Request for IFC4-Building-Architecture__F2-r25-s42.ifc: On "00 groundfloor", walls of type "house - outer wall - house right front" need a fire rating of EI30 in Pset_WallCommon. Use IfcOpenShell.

First a look at what the model holds.

```python
import ifcopenshell
import ifcopenshell.util.element

model = ifcopenshell.open("IFC4-Building-Architecture__F2-r25-s42.ifc")
print(model.schema)
storey = next(s for s in model.by_type("IfcBuildingStorey") if s.Name == "00 groundfloor")
walls = [e for e in ifcopenshell.util.element.get_decomposition(storey) if e.is_a("IfcWall")]
seen = {}
for e in walls:
    element_type = ifcopenshell.util.element.get_type(e)
    key = (element_type.Name if element_type != e and element_type else None, ifcopenshell.util.element.get_pset(e, "Pset_WallCommon", "FireRating"))
    seen[key] = seen.get(key, 0) + 1
for (name, value), count in sorted(seen.items(), key=str):
    print(count, "x", name, "|", value)
```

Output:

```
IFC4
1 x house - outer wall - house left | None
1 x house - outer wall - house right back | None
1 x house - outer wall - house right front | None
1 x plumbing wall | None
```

```python
import ifcopenshell
import ifcopenshell.api.pset
import ifcopenshell.util.element

model = ifcopenshell.open("IFC4-Building-Architecture__F2-r25-s42.ifc")

storey = next(s for s in model.by_type("IfcBuildingStorey") if s.Name == "00 groundfloor")
walls = [e for e in ifcopenshell.util.element.get_decomposition(storey) if e.is_a("IfcWall")]

count = 0
for e in walls:
    element_type = ifcopenshell.util.element.get_type(e)
    if element_type in (None, e) or element_type.Name != "house - outer wall - house right front":
        continue
    # add_pset returns the element's existing set when there is one.
    pset = ifcopenshell.api.pset.add_pset(model, product=e, name="Pset_WallCommon")
    ifcopenshell.api.pset.edit_pset(model, pset=pset, properties={"FireRating": "EI30"})
    count += 1

print(count, "walls updated")

model.write("IFC4-Building-Architecture__F2-r25-s42_v2.ifc")
```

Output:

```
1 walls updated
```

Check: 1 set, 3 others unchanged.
